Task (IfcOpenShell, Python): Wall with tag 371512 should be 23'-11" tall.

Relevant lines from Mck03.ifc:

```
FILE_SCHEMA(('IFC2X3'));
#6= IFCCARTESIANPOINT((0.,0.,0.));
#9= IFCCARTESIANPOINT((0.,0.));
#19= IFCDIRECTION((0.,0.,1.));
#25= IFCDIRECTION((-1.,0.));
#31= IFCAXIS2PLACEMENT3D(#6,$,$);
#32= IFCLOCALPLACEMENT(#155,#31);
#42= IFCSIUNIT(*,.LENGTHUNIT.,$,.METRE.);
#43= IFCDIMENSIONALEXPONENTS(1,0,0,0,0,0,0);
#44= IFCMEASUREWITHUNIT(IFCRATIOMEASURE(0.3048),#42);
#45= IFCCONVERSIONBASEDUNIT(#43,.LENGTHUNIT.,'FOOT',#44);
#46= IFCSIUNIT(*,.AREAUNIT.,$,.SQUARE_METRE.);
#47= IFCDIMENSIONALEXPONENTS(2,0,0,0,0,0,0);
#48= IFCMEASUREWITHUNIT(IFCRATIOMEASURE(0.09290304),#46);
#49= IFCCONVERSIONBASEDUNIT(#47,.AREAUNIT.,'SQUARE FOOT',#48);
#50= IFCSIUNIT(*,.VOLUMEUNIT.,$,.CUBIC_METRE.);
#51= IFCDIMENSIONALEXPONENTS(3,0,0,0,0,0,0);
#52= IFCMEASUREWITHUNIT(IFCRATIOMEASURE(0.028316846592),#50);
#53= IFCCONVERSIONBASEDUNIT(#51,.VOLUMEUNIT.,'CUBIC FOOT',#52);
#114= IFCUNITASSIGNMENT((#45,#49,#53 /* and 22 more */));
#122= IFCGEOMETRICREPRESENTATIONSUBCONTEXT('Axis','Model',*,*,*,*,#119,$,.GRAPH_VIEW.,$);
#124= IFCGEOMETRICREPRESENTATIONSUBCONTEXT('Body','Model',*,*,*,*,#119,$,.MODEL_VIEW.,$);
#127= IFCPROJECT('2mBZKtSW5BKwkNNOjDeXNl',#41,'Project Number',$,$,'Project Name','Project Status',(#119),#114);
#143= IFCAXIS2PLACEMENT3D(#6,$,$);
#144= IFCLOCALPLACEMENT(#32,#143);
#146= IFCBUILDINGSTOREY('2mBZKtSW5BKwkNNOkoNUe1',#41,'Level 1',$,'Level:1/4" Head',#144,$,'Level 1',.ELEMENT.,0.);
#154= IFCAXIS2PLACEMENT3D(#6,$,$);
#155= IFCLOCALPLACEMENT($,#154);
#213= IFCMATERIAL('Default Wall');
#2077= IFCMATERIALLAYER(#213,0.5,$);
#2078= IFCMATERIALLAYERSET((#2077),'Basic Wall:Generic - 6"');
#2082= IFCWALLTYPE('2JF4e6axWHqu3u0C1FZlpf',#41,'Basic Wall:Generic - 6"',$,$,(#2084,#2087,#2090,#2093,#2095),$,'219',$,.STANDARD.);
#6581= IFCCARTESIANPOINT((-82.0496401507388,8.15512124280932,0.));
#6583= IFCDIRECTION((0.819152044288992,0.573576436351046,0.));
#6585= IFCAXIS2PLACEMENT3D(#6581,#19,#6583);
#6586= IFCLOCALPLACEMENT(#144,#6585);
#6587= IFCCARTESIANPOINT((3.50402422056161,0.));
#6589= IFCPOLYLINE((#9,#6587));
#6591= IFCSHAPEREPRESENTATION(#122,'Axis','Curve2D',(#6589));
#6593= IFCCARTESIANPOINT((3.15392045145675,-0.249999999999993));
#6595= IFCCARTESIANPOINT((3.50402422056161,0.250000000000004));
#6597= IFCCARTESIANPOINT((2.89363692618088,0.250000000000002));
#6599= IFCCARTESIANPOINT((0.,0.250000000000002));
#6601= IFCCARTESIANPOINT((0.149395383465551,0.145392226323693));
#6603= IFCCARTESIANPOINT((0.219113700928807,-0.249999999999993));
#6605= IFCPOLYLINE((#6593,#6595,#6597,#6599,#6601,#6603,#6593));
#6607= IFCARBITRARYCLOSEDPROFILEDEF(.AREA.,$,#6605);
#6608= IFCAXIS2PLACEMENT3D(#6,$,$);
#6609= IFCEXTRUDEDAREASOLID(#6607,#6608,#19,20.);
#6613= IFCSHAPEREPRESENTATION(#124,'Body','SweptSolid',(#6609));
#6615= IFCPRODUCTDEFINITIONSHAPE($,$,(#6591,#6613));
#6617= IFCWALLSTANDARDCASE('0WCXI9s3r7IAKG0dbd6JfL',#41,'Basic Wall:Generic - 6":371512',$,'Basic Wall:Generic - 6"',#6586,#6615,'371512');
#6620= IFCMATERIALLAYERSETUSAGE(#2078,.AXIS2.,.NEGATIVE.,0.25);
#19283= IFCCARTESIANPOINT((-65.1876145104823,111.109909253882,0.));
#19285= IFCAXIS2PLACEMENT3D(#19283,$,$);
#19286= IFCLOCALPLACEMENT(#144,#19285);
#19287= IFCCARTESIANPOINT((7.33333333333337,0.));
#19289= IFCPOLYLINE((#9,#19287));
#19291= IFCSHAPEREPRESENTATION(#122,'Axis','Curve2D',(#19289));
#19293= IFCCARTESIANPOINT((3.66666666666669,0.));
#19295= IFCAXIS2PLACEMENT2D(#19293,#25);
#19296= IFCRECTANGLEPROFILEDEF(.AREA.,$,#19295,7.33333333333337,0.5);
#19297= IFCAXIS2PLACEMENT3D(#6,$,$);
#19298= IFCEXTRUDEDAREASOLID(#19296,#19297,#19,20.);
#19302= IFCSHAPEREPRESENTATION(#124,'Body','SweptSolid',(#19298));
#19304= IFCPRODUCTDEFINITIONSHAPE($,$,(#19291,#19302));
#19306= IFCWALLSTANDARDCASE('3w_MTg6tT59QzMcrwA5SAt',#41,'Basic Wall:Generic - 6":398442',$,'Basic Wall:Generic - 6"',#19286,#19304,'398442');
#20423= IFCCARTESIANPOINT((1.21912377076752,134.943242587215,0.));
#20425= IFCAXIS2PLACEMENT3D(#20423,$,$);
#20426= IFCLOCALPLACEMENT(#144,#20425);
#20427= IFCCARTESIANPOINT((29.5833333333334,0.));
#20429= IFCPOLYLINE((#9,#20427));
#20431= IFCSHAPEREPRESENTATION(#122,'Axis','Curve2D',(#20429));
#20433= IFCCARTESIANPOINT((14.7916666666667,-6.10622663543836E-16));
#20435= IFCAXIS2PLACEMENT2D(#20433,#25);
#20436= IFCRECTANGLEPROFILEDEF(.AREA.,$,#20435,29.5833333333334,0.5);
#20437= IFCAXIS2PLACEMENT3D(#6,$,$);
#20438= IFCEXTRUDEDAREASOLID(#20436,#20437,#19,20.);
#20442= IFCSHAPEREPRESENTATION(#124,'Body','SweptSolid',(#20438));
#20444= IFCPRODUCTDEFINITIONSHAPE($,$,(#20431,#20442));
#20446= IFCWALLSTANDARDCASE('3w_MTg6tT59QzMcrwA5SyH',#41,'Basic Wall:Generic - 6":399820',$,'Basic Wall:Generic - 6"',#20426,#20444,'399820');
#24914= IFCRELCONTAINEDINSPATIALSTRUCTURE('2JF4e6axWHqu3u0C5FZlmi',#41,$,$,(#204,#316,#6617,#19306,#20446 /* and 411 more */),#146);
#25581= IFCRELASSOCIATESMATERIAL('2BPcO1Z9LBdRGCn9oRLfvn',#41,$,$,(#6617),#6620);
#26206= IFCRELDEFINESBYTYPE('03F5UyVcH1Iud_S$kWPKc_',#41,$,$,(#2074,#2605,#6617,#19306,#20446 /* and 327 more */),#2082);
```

```python
import ifcopenshell
import ifcopenshell.geom
import ifcopenshell.util.representation
import ifcopenshell.util.shape
import ifcopenshell.util.unit

model = ifcopenshell.open("Mck03.ifc")
unit_scale = ifcopenshell.util.unit.calculate_unit_scale(model)
settings = ifcopenshell.geom.settings()


def volume(element):
    """Net volume in cubic metres, openings subtracted."""
    shape = ifcopenshell.geom.create_shape(settings, element)
    return ifcopenshell.util.shape.get_volume(shape.geometry)


wall = model.by_guid("0WCXI9s3r7IAKG0dbd6JfL")
before = volume(wall)

body = ifcopenshell.util.representation.get_representation(wall, "Model", "Body")
solid = body.Items[0]
old_height = solid.Depth
solid.Depth = 287 * 0.0254 / unit_scale
after = volume(wall)

print(f"height {old_height:g} -> {solid.Depth:g}, volume {before:.3f} -> {after:.3f} m3")

model.write("Mck03-out.ifc")
```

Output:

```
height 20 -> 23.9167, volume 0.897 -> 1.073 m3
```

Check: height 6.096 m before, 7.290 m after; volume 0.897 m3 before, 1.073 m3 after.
